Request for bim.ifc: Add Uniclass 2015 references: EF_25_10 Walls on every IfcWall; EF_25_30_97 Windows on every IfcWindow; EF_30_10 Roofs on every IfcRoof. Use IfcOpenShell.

First a look at what the model holds.

```python
import ifcopenshell

model = ifcopenshell.open("bim.ifc")
print(model.schema)
print("classifications:", [c.Name for c in model.by_type("IfcClassification")])
for ifc_class in ("IfcDoor", "IfcRoof", "IfcStair", "IfcWall", "IfcWindow"):
    print(ifc_class, len(model.by_type(ifc_class)))
```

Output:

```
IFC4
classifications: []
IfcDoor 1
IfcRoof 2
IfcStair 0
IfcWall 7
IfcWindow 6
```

```python
import ifcopenshell
import ifcopenshell.api.classification

model = ifcopenshell.open("bim.ifc")

system = ifcopenshell.api.classification.add_classification(model, classification="Uniclass 2015")

codes = {
    "IfcWall": ("EF_25_10", "Walls"),
    "IfcWindow": ("EF_25_30_97", "Windows"),
    "IfcRoof": ("EF_30_10", "Roofs"),
}
for ifc_class, (code, name) in codes.items():
    products = model.by_type(ifc_class)
    ifcopenshell.api.classification.add_reference(
        model, products=products, classification=system, identification=code, name=name
    )
    print(code, len(products))

model.write("bim-out.ifc")
```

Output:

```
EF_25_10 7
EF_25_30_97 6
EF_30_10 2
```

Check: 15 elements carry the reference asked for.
